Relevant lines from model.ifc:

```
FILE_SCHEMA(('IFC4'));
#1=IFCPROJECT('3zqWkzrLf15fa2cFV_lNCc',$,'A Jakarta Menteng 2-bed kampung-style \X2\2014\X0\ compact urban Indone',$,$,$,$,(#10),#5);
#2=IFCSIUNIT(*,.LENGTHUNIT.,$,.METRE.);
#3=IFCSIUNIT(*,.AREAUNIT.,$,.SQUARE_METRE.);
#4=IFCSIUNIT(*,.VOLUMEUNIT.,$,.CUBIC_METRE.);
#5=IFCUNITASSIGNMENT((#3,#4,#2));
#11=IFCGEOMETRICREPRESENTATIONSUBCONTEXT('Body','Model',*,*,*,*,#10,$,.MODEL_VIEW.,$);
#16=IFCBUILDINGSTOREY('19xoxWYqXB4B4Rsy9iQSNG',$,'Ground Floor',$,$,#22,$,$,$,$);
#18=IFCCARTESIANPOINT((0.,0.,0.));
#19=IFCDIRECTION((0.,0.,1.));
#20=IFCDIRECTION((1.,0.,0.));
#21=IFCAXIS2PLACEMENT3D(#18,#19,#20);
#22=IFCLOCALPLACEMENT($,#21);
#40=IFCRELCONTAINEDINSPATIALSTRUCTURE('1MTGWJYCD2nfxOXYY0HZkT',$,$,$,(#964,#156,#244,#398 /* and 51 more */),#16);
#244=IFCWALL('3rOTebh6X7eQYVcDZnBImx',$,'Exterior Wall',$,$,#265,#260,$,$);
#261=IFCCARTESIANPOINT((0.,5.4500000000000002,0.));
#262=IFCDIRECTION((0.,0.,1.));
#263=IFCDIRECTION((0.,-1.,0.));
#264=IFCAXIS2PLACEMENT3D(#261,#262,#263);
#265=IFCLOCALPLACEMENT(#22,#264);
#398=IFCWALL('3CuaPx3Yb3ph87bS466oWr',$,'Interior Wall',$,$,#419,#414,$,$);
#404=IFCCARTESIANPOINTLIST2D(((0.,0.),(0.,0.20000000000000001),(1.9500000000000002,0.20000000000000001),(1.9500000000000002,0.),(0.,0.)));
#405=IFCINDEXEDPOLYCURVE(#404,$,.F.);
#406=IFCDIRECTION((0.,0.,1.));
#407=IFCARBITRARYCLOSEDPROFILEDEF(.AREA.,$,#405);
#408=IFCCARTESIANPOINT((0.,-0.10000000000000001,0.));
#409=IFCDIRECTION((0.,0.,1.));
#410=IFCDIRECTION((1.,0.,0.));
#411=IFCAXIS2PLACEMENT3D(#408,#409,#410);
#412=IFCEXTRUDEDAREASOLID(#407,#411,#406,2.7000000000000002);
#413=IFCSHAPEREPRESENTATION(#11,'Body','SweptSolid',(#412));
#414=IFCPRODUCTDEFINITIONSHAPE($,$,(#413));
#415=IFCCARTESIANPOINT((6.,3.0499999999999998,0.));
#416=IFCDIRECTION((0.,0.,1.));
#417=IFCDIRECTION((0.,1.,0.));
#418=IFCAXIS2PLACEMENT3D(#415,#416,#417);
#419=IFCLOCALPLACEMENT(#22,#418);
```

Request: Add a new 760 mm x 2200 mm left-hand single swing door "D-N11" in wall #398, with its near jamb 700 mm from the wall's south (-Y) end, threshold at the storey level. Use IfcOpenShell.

```python
import numpy as np
import ifcopenshell
import ifcopenshell.api.feature
import ifcopenshell.api.geometry
import ifcopenshell.api.root
import ifcopenshell.api.spatial
import ifcopenshell.geom
import ifcopenshell.util.element
import ifcopenshell.util.placement
import ifcopenshell.util.representation
import ifcopenshell.util.shape
import ifcopenshell.util.unit

model = ifcopenshell.open("model.ifc")
unit_scale = ifcopenshell.util.unit.calculate_unit_scale(model)
settings = ifcopenshell.geom.settings()


def volume(element):
    """Net volume in cubic metres, openings subtracted."""
    shape = ifcopenshell.geom.create_shape(settings, element)
    return ifcopenshell.util.shape.get_volume(shape.geometry)


wall = model.by_guid("3CuaPx3Yb3ph87bS466oWr")
storey = ifcopenshell.util.element.get_container(wall, ifc_class="IfcBuildingStorey")
context = ifcopenshell.util.representation.get_context(model, "Model", "Body", "MODEL_VIEW")
before = volume(wall)

width, height, from_end, sill = 0.76, 2.2, 0.7, 0.0  # metres

# The wall runs along its own X axis, and the end named is its -X end.
wall_shape = ifcopenshell.geom.create_shape(settings, wall)
x, y, z = ifcopenshell.util.shape.get_vertices(wall_shape.geometry).T
start = x.min() + from_end
face, thickness = float(y.min()), float(y.max() - y.min())
wall_matrix = ifcopenshell.util.placement.get_local_placement(wall.ObjectPlacement)
level = ifcopenshell.util.placement.get_local_placement(storey.ObjectPlacement)[2, 3]


def in_wall(x, y):
    """Placement at x, y metres in the wall's axes, at sill height."""
    matrix = wall_matrix.copy()
    matrix[:, 3] = wall_matrix @ np.array([x / unit_scale, y / unit_scale, 0.0, 1.0])
    matrix[2, 3] = level + sill / unit_scale
    return matrix


# Opening: a box that overshoots both wall faces by 50 mm.
opening = ifcopenshell.api.root.create_entity(model, ifc_class="IfcOpeningElement", predefined_type="OPENING")
box = ifcopenshell.api.geometry.add_wall_representation(
    model, context=context, length=width, height=height, thickness=thickness + 0.1
)
ifcopenshell.api.geometry.assign_representation(model, product=opening, representation=box)
ifcopenshell.api.geometry.edit_object_placement(model, product=opening, matrix=in_wall(start, face - 0.05), is_si=False)
ifcopenshell.api.feature.add_feature(model, feature=opening, element=wall)

door = ifcopenshell.api.root.create_entity(model, ifc_class="IfcDoor", name="D-N11", predefined_type="DOOR")
door.OverallWidth, door.OverallHeight = width / unit_scale, height / unit_scale
door.OperationType = "SINGLE_SWING_LEFT"
body = ifcopenshell.api.geometry.add_door_representation(
    model,
    context=context,
    overall_width=door.OverallWidth,
    overall_height=door.OverallHeight,
    operation_type="SINGLE_SWING_LEFT",
    lining_properties={"LiningDepth": thickness / unit_scale, "ThresholdDepth": thickness / unit_scale},
)
ifcopenshell.api.geometry.assign_representation(model, product=door, representation=body)
ifcopenshell.api.spatial.assign_container(model, products=[door], relating_structure=storey)
ifcopenshell.api.feature.add_filling(model, opening=opening, element=door)

# The lining spans the wall, so the door starts at the wall face.
ifcopenshell.api.geometry.edit_object_placement(model, product=door, matrix=in_wall(start, face), is_si=False)

after = volume(wall)

print(f"wall volume {before:.3f} -> {after:.3f} m3")

model.write("model_updated.ifc")
```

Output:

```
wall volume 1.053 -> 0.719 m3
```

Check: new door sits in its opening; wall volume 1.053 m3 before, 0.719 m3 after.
